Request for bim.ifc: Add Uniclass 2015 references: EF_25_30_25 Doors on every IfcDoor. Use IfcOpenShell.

First a look at what the model holds.

```python
import ifcopenshell

model = ifcopenshell.open("bim.ifc")
print(model.schema)
print("classifications:", [c.Name for c in model.by_type("IfcClassification")])
for ifc_class in ("IfcDoor", "IfcRoof", "IfcStair", "IfcWall", "IfcWindow"):
    print(ifc_class, len(model.by_type(ifc_class)))
```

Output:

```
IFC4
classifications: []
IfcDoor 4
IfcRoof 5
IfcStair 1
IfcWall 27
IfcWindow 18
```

```python
import ifcopenshell
import ifcopenshell.api.classification

model = ifcopenshell.open("bim.ifc")

system = ifcopenshell.api.classification.add_classification(model, classification="Uniclass 2015")

codes = {
    "IfcDoor": ("EF_25_30_25", "Doors"),
}
for ifc_class, (code, name) in codes.items():
    products = model.by_type(ifc_class)
    ifcopenshell.api.classification.add_reference(
        model, products=products, classification=system, identification=code, name=name
    )
    print(code, len(products))

model.write("bim-out.ifc")
```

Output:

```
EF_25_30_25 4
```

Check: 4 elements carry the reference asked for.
